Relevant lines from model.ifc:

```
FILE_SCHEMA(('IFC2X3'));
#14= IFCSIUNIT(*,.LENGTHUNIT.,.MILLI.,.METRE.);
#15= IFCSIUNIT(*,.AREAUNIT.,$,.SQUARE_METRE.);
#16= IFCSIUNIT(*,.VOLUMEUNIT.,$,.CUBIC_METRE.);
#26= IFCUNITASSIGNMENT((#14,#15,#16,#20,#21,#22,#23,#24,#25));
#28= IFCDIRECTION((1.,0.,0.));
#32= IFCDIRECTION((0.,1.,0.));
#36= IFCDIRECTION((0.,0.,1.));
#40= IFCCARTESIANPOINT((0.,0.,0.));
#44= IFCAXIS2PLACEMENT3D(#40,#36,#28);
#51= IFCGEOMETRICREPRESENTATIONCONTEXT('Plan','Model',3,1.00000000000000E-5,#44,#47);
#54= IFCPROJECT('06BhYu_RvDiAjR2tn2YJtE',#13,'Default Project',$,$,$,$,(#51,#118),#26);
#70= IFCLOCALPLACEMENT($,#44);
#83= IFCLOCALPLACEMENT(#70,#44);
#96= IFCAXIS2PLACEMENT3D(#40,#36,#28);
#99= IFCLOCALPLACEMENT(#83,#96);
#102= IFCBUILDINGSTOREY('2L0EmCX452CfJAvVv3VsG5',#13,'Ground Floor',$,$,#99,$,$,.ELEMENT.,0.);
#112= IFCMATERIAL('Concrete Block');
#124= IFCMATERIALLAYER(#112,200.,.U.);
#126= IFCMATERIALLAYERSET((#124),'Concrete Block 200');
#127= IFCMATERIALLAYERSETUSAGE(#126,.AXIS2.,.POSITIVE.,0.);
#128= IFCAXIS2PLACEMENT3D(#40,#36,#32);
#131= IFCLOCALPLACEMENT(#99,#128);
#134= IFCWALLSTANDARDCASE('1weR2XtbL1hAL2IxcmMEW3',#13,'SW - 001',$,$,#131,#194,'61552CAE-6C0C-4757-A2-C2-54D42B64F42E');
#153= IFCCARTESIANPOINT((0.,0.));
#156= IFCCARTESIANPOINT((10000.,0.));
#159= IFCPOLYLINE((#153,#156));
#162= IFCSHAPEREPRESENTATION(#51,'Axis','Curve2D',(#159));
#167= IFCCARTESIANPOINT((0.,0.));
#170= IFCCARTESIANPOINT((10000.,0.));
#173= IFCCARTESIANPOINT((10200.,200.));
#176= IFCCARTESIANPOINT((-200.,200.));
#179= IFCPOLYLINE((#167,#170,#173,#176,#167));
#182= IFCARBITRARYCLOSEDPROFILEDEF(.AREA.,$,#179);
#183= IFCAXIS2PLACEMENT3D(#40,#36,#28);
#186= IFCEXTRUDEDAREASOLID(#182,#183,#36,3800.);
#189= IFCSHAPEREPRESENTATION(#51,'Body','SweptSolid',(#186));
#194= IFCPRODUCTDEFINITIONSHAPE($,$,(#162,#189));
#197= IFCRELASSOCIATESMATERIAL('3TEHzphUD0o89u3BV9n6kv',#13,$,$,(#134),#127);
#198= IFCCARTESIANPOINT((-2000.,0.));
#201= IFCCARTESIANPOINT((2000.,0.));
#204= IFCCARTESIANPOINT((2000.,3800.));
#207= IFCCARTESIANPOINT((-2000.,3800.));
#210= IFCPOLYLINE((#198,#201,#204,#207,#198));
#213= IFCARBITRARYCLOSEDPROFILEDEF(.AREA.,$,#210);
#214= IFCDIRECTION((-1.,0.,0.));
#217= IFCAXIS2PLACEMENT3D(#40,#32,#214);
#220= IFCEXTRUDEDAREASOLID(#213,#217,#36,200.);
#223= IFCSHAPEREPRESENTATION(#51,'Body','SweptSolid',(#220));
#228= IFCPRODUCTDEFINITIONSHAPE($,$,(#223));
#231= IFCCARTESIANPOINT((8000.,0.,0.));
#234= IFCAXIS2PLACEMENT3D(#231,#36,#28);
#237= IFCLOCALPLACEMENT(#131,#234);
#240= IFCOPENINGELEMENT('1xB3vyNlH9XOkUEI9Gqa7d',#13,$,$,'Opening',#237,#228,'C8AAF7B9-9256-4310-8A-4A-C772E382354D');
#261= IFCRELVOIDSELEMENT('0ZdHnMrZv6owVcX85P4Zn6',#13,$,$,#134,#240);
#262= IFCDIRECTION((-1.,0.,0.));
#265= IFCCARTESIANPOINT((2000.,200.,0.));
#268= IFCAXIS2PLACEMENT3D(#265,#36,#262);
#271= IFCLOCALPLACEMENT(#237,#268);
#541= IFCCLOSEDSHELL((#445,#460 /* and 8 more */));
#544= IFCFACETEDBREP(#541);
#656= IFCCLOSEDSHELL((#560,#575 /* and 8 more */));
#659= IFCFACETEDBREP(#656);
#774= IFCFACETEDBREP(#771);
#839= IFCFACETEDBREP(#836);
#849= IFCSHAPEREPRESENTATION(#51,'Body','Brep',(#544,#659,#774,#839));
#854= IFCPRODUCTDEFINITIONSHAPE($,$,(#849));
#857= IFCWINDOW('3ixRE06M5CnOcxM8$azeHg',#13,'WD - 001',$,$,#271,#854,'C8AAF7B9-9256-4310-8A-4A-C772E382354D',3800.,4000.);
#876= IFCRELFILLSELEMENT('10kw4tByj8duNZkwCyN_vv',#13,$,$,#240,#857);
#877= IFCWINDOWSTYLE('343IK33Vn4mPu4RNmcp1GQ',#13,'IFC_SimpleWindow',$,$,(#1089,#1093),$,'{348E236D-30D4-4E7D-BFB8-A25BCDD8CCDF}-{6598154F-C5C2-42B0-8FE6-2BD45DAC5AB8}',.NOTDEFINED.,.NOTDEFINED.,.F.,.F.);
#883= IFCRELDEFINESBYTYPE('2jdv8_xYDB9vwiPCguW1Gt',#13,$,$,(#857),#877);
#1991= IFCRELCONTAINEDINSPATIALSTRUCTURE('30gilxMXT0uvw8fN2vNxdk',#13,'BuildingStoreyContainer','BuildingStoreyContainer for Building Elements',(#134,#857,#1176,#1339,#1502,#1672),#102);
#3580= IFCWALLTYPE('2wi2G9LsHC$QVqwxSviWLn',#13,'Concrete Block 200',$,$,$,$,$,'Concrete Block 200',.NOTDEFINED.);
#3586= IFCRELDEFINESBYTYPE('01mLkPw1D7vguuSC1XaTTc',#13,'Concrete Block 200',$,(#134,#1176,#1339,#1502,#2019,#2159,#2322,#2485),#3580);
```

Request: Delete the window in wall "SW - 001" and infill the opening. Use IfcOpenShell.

```python
import ifcopenshell
import ifcopenshell.api.feature
import ifcopenshell.api.root
import ifcopenshell.geom
import ifcopenshell.util.shape

model = ifcopenshell.open("model.ifc")
settings = ifcopenshell.geom.settings()


def volume(element):
    """Net volume in cubic metres, openings subtracted."""
    shape = ifcopenshell.geom.create_shape(settings, element)
    return ifcopenshell.util.shape.get_volume(shape.geometry)


window = model.by_guid("3ixRE06M5CnOcxM8$azeHg")
opening = window.FillsVoids[0].RelatingOpeningElement
wall = opening.VoidsElements[0].RelatingBuildingElement
before = volume(wall)

ifcopenshell.api.root.remove_product(model, product=window)
ifcopenshell.api.feature.remove_feature(model, feature=opening)

after = volume(wall)

print(f"wall volume {before:.3f} -> {after:.3f} m3")

model.write("model_edited.ifc")
```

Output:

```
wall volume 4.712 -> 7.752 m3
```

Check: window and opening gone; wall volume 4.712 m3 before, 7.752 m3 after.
